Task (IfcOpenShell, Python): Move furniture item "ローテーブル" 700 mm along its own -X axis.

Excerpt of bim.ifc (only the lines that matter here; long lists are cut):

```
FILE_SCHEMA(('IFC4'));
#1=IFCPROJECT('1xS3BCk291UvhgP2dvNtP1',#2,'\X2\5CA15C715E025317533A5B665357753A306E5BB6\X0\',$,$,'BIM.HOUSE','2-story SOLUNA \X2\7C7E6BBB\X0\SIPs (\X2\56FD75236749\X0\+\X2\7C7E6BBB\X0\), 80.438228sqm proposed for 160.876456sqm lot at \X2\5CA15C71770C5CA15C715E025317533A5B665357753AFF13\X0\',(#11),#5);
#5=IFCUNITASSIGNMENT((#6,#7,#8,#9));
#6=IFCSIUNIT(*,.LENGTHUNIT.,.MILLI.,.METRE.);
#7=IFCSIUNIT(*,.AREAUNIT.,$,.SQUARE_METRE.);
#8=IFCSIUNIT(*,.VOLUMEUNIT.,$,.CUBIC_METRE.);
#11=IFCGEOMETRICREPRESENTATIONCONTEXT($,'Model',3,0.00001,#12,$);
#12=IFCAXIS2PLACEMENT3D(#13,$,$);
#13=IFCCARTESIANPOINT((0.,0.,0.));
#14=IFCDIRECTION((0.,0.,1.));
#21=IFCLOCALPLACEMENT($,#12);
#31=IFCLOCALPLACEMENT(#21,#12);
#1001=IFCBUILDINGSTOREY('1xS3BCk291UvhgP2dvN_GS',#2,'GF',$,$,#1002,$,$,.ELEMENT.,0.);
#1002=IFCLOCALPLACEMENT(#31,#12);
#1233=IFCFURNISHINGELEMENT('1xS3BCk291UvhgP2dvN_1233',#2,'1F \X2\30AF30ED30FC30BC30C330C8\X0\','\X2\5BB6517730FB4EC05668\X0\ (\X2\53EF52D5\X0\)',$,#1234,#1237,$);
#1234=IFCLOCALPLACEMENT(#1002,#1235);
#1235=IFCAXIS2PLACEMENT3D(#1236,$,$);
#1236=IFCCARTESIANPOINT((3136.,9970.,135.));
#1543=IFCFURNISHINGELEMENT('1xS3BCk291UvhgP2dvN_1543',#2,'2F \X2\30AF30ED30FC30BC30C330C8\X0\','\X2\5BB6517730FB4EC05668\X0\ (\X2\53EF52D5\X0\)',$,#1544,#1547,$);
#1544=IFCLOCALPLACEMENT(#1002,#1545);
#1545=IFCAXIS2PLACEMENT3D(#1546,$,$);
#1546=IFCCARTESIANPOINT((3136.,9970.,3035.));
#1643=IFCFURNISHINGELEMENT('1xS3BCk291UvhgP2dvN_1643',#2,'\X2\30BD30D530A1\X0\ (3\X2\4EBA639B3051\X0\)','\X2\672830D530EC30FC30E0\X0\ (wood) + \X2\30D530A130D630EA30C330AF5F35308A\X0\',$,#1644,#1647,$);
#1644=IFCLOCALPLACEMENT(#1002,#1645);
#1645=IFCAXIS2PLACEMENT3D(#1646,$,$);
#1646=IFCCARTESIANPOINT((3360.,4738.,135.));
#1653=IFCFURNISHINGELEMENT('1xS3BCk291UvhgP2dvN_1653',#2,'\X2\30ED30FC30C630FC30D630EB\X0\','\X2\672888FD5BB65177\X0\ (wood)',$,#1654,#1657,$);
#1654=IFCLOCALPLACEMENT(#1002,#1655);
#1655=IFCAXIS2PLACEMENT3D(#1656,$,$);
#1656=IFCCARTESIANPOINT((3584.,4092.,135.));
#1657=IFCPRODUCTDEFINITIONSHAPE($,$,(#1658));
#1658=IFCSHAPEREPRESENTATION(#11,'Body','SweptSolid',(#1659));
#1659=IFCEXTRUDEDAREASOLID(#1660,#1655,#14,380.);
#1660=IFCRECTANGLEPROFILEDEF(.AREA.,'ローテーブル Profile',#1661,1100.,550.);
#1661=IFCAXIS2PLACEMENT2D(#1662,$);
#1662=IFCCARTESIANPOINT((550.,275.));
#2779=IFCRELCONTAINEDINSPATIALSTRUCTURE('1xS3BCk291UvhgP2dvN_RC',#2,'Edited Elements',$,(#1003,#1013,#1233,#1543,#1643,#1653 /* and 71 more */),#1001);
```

```python
import ifcopenshell
import ifcopenshell.api.geometry
import ifcopenshell.util.placement
import ifcopenshell.util.unit

model = ifcopenshell.open("bim.ifc")
unit_scale = ifcopenshell.util.unit.calculate_unit_scale(model)

item = model.by_id(1653)
matrix = ifcopenshell.util.placement.get_local_placement(item.ObjectPlacement)
matrix[:3, 3] -= matrix[:3, 0] * 0.7 / unit_scale
ifcopenshell.api.geometry.edit_object_placement(model, product=item, matrix=matrix, is_si=False)

print(ifcopenshell.util.placement.get_local_placement(item.ObjectPlacement).round(3) + 0.0)

model.write("bim_edited.ifc")
```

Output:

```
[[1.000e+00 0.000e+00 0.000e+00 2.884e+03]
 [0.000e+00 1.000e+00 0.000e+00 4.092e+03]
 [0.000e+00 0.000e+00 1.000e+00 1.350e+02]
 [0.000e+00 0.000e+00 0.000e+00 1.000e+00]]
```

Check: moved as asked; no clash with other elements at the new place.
